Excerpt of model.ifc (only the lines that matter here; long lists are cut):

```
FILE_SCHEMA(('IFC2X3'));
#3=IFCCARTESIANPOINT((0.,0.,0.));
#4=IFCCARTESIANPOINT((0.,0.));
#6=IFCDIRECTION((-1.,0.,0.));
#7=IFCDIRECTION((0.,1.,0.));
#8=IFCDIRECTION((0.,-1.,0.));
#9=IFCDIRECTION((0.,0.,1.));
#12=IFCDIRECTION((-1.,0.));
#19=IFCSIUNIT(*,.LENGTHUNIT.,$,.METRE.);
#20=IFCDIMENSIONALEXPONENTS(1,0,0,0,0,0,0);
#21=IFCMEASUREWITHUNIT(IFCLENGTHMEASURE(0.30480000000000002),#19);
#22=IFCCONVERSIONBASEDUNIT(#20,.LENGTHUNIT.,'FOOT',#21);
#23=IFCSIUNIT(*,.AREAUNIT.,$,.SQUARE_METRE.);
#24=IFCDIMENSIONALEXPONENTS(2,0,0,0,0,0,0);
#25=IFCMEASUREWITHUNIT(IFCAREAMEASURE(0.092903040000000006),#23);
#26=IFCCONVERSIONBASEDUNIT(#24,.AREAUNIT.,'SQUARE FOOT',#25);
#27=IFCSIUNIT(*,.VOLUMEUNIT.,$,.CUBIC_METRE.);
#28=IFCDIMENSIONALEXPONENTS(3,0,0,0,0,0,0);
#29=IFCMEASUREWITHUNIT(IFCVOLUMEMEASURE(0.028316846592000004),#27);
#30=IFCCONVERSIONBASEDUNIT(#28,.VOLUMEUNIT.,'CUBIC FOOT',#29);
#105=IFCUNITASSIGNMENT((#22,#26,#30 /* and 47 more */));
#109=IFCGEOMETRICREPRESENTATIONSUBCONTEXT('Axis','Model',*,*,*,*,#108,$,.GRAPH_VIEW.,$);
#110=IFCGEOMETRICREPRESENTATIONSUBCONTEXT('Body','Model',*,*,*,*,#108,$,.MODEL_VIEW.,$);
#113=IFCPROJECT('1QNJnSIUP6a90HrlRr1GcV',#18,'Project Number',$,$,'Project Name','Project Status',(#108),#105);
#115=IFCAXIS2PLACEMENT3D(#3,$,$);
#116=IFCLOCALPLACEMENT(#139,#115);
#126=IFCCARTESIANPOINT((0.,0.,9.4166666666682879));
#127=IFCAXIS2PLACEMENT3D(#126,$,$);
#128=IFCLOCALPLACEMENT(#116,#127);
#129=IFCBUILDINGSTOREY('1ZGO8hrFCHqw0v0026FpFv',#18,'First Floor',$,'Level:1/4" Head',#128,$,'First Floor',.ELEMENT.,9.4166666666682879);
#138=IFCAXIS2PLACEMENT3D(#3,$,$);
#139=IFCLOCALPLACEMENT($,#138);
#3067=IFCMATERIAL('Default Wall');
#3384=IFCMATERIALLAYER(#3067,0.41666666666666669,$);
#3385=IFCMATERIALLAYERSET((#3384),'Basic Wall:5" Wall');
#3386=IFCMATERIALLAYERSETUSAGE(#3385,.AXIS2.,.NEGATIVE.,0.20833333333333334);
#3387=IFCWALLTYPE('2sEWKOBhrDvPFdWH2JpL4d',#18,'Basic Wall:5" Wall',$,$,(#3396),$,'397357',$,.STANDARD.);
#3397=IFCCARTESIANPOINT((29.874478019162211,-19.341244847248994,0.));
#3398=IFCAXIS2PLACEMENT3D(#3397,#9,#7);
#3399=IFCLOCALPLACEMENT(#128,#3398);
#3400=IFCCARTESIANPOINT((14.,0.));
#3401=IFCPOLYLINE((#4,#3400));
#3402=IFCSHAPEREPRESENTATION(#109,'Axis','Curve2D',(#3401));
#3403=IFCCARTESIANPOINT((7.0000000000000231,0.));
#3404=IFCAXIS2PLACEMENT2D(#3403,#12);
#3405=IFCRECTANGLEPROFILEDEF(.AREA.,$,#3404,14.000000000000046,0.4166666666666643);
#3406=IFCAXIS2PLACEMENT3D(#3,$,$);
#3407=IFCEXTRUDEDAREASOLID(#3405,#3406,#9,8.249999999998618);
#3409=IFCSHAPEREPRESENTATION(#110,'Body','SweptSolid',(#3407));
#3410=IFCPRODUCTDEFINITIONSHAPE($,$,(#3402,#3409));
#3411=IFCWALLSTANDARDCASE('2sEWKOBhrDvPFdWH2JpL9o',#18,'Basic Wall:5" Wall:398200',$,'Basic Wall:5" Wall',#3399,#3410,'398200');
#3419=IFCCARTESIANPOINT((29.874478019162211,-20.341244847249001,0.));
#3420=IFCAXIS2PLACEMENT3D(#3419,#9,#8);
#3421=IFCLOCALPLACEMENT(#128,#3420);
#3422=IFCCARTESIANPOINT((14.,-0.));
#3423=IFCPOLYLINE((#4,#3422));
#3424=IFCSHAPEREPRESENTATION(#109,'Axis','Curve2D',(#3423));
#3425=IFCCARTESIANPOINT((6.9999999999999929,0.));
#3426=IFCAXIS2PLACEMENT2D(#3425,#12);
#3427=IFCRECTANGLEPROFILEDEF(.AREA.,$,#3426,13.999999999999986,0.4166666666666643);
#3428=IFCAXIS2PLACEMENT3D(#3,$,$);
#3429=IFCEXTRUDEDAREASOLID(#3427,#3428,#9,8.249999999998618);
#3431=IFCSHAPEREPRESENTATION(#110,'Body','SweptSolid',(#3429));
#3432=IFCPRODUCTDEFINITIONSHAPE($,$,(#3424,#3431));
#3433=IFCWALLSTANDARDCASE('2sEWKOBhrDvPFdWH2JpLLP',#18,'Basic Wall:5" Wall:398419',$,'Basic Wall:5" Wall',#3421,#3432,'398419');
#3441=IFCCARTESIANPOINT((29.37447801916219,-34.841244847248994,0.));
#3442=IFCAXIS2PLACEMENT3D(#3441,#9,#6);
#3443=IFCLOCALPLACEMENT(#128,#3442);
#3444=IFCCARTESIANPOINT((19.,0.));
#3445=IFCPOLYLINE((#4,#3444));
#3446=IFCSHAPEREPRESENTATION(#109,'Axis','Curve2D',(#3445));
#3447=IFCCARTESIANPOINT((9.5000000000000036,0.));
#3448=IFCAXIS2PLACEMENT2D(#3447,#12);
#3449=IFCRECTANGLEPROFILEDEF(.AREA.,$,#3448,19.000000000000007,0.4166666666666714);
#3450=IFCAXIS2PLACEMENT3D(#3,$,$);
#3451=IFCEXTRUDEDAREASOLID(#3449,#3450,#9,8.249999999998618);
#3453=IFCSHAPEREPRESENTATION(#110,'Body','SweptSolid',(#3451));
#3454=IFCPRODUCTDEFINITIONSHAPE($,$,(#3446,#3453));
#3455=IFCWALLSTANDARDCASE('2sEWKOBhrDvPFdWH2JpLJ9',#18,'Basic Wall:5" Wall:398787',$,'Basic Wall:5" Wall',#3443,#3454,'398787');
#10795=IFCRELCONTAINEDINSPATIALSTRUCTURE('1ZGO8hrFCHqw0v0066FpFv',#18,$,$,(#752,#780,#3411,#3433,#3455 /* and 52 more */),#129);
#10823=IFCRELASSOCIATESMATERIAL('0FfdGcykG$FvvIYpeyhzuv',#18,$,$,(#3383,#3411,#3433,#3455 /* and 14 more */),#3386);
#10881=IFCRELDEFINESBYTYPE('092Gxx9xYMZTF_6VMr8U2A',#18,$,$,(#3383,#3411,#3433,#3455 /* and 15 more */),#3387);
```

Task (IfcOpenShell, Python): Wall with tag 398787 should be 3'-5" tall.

```python
import ifcopenshell
import ifcopenshell.geom
import ifcopenshell.util.representation
import ifcopenshell.util.shape
import ifcopenshell.util.unit

model = ifcopenshell.open("model.ifc")
unit_scale = ifcopenshell.util.unit.calculate_unit_scale(model)
settings = ifcopenshell.geom.settings()


def volume(element):
    """Net volume in cubic metres, openings subtracted."""
    shape = ifcopenshell.geom.create_shape(settings, element)
    return ifcopenshell.util.shape.get_volume(shape.geometry)


wall = model.by_guid("2sEWKOBhrDvPFdWH2JpLJ9")
before = volume(wall)

body = ifcopenshell.util.representation.get_representation(wall, "Model", "Body")
solid = body.Items[0]
old_height = solid.Depth
solid.Depth = 41 * 0.0254 / unit_scale
after = volume(wall)

print(f"height {old_height:g} -> {solid.Depth:g}, volume {before:.3f} -> {after:.3f} m3")

model.write("model_edited.ifc")
```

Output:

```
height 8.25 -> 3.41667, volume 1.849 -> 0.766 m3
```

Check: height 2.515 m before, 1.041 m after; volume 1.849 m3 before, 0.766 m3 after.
